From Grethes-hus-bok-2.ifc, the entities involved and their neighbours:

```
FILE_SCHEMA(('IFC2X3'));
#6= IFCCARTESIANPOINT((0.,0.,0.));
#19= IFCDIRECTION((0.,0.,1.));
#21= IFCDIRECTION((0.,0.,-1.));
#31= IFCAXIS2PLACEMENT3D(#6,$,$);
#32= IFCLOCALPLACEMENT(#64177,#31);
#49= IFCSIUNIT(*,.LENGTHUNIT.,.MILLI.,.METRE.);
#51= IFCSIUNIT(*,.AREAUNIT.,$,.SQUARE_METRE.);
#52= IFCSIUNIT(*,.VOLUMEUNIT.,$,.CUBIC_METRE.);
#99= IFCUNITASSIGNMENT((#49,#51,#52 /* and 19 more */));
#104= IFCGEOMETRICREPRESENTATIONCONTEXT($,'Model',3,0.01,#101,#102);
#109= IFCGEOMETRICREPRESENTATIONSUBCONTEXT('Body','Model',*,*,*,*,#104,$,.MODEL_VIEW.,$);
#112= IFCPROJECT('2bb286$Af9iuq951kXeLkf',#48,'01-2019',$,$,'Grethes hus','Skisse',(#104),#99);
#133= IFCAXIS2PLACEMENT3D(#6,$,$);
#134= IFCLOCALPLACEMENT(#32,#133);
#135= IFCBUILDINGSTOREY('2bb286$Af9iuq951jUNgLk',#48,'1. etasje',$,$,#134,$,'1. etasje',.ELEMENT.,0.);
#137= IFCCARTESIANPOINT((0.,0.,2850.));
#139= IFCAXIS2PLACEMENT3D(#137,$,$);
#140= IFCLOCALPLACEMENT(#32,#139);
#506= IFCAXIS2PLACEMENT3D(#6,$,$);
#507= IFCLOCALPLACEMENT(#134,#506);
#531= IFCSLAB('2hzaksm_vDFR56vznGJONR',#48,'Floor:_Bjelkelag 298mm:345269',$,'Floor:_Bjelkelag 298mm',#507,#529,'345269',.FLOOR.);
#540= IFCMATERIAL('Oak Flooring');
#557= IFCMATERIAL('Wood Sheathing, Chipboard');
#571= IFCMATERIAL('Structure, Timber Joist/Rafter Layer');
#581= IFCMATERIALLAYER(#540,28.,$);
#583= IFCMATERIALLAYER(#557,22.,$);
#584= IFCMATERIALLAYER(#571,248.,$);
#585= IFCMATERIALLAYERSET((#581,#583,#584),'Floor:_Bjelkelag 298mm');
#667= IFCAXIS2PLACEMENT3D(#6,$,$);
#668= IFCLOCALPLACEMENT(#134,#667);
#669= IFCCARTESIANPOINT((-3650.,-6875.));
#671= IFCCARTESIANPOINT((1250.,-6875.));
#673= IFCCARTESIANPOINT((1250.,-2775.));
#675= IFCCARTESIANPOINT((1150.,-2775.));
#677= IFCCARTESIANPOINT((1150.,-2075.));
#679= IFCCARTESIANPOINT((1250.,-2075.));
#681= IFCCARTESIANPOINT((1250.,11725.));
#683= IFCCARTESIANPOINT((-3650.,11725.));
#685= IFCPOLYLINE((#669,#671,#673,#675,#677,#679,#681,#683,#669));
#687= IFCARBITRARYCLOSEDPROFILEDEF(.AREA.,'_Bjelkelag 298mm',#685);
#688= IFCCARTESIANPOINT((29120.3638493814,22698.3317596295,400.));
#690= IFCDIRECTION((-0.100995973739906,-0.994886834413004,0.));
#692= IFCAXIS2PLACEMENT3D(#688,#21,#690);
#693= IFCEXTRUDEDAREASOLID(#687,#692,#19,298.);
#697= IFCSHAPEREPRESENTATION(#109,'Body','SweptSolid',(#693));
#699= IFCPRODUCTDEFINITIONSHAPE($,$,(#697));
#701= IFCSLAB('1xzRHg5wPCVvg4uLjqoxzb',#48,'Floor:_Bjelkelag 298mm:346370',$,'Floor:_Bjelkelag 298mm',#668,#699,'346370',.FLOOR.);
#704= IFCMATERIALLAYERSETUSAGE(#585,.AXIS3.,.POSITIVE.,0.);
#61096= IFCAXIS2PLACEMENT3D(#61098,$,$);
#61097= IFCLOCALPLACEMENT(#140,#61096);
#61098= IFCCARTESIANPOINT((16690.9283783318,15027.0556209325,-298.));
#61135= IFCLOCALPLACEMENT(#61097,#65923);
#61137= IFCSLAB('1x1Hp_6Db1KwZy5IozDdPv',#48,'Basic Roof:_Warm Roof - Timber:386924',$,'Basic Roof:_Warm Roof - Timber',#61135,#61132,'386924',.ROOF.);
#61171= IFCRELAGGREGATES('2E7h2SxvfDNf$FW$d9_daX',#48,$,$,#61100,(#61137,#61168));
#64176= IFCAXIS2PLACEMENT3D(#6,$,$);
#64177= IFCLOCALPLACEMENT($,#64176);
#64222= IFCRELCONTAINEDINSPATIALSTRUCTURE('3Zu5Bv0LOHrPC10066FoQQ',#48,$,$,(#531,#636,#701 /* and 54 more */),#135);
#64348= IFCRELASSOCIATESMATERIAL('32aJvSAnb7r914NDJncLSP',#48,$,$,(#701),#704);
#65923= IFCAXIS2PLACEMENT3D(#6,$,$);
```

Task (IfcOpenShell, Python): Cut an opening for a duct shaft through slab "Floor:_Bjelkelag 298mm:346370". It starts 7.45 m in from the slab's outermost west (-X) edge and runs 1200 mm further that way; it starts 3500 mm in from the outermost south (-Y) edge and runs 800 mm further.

```python
import numpy as np
import ifcopenshell
import ifcopenshell.api.feature
import ifcopenshell.api.geometry
import ifcopenshell.api.root
import ifcopenshell.geom
import ifcopenshell.util.placement
import ifcopenshell.util.representation
import ifcopenshell.util.shape
import ifcopenshell.util.unit

model = ifcopenshell.open("Grethes-hus-bok-2.ifc")
unit_scale = ifcopenshell.util.unit.calculate_unit_scale(model)
settings = ifcopenshell.geom.settings()


def volume(element):
    """Net volume in cubic metres, openings subtracted."""
    shape = ifcopenshell.geom.create_shape(settings, element)
    return ifcopenshell.util.shape.get_volume(shape.geometry)


slab = model.by_guid("1xzRHg5wPCVvg4uLjqoxzb")
before = volume(slab)

# Extent in the slab's own axes, in metres. The edges named are its -X and -Y sides.
slab_shape = ifcopenshell.geom.create_shape(settings, slab)
vertices = ifcopenshell.util.shape.get_vertices(slab_shape.geometry)
x_min, y_min, bottom = vertices.min(axis=0)
top = vertices[:, 2].max()

opening = ifcopenshell.api.root.create_entity(model, ifc_class="IfcOpeningElement", name="Duct shaft opening")
context = ifcopenshell.util.representation.get_context(model, "Model", "Body", "MODEL_VIEW")
width, depth = 1.2, 0.8
outline = [(0.0, 0.0), (width, 0.0), (width, depth), (0.0, depth), (0.0, 0.0)]
# Overshoot both faces by 50 mm so the cut is clean.
shape = ifcopenshell.api.geometry.add_slab_representation(
    model, context=context, depth=top - bottom + 0.1, polyline=outline
)
ifcopenshell.api.geometry.assign_representation(model, product=opening, representation=shape)

matrix = ifcopenshell.util.placement.get_local_placement(slab.ObjectPlacement)
matrix[:, 3] = matrix @ np.append(np.array([x_min + 7.45, y_min + 3.5, bottom - 0.05]) / unit_scale, 1.0)
ifcopenshell.api.geometry.edit_object_placement(model, product=opening, matrix=matrix, is_si=False)
ifcopenshell.api.feature.add_feature(model, feature=opening, element=slab)

after = volume(slab)

print(f"slab volume {before:.3f} -> {after:.3f} m3")

model.write("Grethes-hus-bok-2_v2.ifc")
```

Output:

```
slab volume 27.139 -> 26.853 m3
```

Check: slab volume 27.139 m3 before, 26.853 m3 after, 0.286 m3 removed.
